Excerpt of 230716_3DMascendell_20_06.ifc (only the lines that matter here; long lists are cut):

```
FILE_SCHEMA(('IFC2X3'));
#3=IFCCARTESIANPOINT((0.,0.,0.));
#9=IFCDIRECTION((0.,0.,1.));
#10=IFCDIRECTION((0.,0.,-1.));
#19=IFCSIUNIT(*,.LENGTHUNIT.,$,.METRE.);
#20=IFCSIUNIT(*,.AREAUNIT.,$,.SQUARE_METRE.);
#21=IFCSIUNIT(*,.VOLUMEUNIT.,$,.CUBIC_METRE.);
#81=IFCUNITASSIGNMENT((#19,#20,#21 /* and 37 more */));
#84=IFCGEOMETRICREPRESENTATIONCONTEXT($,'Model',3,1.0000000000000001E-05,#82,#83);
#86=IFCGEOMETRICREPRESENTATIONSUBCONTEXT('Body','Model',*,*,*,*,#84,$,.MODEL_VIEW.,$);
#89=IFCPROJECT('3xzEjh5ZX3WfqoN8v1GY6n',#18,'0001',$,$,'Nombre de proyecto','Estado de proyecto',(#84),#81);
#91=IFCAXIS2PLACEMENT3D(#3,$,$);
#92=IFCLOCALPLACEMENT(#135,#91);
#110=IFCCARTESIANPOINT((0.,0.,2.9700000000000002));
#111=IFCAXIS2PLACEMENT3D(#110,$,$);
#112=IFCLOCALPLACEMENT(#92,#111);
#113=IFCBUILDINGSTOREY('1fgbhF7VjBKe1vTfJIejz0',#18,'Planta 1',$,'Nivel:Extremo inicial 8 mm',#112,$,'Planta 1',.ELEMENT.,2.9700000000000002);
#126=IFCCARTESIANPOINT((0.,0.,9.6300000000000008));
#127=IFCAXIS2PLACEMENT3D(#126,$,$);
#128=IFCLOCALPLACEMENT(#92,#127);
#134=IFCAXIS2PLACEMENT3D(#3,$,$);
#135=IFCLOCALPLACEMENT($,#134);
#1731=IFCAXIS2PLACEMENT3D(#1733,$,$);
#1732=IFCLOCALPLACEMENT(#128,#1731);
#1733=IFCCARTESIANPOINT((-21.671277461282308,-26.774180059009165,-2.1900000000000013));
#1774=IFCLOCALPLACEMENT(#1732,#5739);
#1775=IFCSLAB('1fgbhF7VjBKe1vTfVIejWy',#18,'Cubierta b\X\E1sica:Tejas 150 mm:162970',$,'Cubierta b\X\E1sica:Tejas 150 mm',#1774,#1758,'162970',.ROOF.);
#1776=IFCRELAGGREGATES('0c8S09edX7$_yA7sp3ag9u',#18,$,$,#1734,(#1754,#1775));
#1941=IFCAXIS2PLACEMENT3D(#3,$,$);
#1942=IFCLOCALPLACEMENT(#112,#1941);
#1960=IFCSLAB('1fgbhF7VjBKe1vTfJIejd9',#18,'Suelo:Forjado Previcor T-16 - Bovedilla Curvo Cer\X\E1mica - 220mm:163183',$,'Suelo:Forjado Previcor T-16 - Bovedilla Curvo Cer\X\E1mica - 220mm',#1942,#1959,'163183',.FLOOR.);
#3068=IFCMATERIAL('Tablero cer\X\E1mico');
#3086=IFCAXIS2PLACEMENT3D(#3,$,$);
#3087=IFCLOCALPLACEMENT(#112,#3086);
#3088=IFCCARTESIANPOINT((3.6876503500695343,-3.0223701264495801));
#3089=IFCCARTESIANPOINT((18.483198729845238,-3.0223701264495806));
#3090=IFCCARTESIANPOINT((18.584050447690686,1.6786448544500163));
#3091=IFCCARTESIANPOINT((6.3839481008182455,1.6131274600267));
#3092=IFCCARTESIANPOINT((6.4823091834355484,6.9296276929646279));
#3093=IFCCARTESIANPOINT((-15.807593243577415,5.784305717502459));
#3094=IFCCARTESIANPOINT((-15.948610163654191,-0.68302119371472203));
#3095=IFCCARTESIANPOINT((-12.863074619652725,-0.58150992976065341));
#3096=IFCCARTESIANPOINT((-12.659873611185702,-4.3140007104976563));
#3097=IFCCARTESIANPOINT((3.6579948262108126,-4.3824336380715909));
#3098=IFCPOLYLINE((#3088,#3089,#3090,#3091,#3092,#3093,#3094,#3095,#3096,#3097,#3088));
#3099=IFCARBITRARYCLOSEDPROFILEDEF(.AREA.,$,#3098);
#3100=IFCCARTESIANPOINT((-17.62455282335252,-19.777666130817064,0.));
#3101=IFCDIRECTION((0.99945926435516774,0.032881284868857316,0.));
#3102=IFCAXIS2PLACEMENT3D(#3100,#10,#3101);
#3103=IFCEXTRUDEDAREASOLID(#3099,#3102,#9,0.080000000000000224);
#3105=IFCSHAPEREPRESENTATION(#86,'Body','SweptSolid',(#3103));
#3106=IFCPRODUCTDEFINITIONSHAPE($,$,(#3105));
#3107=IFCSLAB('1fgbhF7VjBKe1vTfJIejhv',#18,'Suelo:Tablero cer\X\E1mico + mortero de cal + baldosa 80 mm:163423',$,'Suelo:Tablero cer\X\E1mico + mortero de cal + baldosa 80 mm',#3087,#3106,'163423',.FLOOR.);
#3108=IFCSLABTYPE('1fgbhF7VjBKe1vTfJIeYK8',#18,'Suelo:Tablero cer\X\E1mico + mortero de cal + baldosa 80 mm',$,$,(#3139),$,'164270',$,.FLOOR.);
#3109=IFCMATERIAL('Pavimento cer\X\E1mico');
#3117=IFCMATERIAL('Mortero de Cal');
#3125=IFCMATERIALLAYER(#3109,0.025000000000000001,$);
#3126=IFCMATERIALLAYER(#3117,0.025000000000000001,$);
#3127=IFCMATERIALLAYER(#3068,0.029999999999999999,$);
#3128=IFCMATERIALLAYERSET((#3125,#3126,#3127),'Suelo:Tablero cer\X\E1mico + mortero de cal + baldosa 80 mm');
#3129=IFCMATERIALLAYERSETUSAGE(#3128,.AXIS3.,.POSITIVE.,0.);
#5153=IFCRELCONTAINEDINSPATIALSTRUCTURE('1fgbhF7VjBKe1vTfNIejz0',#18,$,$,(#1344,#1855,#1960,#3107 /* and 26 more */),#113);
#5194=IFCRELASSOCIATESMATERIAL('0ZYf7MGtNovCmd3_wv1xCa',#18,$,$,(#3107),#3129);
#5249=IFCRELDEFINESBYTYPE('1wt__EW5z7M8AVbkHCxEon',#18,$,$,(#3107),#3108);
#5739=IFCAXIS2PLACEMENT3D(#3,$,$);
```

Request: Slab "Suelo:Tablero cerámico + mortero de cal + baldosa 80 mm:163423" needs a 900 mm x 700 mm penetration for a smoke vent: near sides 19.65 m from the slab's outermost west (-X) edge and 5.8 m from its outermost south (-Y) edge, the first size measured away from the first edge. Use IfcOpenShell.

```python
import numpy as np
import ifcopenshell
import ifcopenshell.api.feature
import ifcopenshell.api.geometry
import ifcopenshell.api.root
import ifcopenshell.geom
import ifcopenshell.util.placement
import ifcopenshell.util.representation
import ifcopenshell.util.shape
import ifcopenshell.util.unit

model = ifcopenshell.open("230716_3DMascendell_20_06.ifc")
unit_scale = ifcopenshell.util.unit.calculate_unit_scale(model)
settings = ifcopenshell.geom.settings()


def volume(element):
    """Net volume in cubic metres, openings subtracted."""
    shape = ifcopenshell.geom.create_shape(settings, element)
    return ifcopenshell.util.shape.get_volume(shape.geometry)


slab = model.by_guid("1fgbhF7VjBKe1vTfJIejhv")
before = volume(slab)

# Extent in the slab's own axes, in metres. The edges named are its -X and -Y sides.
slab_shape = ifcopenshell.geom.create_shape(settings, slab)
vertices = ifcopenshell.util.shape.get_vertices(slab_shape.geometry)
x_min, y_min, bottom = vertices.min(axis=0)
top = vertices[:, 2].max()

opening = ifcopenshell.api.root.create_entity(model, ifc_class="IfcOpeningElement", name="Smoke vent opening")
context = ifcopenshell.util.representation.get_context(model, "Model", "Body", "MODEL_VIEW")
width, depth = 0.9, 0.7
outline = [(0.0, 0.0), (width, 0.0), (width, depth), (0.0, depth), (0.0, 0.0)]
# Overshoot both faces by 50 mm so the cut is clean.
shape = ifcopenshell.api.geometry.add_slab_representation(
    model, context=context, depth=top - bottom + 0.1, polyline=outline
)
ifcopenshell.api.geometry.assign_representation(model, product=opening, representation=shape)

matrix = ifcopenshell.util.placement.get_local_placement(slab.ObjectPlacement)
matrix[:, 3] = matrix @ np.append(np.array([x_min + 19.65, y_min + 5.8, bottom - 0.05]) / unit_scale, 1.0)
ifcopenshell.api.geometry.edit_object_placement(model, product=opening, matrix=matrix, is_si=False)
ifcopenshell.api.feature.add_feature(model, feature=opening, element=slab)

after = volume(slab)

print(f"slab volume {before:.3f} -> {after:.3f} m3")

model.write("230716_3DMascendell_20_06-out.ifc")
```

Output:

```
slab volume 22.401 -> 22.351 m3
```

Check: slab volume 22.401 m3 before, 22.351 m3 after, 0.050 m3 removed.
